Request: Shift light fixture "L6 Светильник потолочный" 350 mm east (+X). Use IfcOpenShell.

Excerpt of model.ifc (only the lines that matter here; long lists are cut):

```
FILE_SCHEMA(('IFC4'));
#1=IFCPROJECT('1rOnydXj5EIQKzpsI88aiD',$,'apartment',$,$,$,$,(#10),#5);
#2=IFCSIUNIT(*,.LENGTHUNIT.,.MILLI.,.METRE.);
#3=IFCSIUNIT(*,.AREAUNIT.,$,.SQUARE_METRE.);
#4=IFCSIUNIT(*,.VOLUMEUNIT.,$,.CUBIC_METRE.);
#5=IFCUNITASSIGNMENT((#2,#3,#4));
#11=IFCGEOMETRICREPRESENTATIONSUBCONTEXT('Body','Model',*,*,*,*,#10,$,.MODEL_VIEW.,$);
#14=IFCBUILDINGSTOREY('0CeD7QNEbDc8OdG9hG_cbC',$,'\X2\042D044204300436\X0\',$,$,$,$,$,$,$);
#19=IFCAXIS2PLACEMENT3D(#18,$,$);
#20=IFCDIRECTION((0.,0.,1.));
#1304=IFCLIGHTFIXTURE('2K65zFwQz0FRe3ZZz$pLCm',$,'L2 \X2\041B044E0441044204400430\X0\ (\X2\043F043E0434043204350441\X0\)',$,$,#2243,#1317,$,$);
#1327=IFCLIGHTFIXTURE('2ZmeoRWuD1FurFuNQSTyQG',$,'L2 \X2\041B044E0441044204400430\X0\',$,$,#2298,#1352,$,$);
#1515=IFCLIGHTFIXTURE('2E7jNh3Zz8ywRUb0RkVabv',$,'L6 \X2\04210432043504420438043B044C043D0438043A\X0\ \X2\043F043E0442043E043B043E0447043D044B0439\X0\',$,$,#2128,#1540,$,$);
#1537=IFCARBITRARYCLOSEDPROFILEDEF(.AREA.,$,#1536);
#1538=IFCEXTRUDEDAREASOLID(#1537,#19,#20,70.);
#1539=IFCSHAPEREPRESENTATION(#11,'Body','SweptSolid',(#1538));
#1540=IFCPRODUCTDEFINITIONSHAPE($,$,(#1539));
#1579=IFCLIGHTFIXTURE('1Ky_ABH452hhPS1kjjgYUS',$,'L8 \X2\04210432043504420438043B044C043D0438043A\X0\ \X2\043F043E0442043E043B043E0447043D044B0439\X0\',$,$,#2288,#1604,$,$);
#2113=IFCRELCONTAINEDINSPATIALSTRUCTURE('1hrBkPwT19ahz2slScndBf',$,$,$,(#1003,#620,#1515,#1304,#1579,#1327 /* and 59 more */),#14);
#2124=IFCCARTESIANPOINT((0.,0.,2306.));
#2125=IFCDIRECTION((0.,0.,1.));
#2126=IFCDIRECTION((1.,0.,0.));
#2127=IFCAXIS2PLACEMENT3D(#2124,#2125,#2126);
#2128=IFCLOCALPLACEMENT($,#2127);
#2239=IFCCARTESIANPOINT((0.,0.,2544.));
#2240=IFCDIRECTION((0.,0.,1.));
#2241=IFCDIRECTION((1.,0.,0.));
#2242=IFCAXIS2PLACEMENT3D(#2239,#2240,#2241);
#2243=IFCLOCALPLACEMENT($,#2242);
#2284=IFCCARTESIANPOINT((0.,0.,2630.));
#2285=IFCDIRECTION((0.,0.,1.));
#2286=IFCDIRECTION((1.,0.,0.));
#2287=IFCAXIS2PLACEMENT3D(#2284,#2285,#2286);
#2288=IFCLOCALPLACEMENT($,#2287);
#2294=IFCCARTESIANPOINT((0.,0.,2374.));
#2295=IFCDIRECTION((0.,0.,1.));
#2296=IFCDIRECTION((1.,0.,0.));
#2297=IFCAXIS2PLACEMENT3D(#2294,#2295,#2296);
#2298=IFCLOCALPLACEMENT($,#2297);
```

```python
import ifcopenshell
import ifcopenshell.api.geometry
import ifcopenshell.util.placement
import ifcopenshell.util.unit

model = ifcopenshell.open("model.ifc")
unit_scale = ifcopenshell.util.unit.calculate_unit_scale(model)

item = model.by_id(1515)
matrix = ifcopenshell.util.placement.get_local_placement(item.ObjectPlacement)
matrix[0, 3] += 0.35 / unit_scale
ifcopenshell.api.geometry.edit_object_placement(model, product=item, matrix=matrix, is_si=False)

print(ifcopenshell.util.placement.get_local_placement(item.ObjectPlacement).round(3) + 0.0)

model.write("model_edited.ifc")
```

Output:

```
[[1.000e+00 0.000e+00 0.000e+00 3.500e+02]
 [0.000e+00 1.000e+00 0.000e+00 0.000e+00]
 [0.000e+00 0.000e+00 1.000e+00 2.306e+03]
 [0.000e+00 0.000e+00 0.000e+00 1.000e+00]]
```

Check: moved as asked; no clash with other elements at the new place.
